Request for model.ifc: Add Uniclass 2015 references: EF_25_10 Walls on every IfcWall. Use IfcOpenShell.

First a look at what the model holds.

```python
import ifcopenshell

model = ifcopenshell.open("model.ifc")
print(model.schema)
print("classifications:", [c.Name for c in model.by_type("IfcClassification")])
for ifc_class in ("IfcDoor", "IfcRoof", "IfcStair", "IfcWall", "IfcWindow"):
    print(ifc_class, len(model.by_type(ifc_class)))
```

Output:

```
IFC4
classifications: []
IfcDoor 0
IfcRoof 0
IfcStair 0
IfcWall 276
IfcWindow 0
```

```python
import ifcopenshell
import ifcopenshell.api.classification

model = ifcopenshell.open("model.ifc")

system = ifcopenshell.api.classification.add_classification(model, classification="Uniclass 2015")

codes = {
    "IfcWall": ("EF_25_10", "Walls"),
}
for ifc_class, (code, name) in codes.items():
    products = model.by_type(ifc_class)
    ifcopenshell.api.classification.add_reference(
        model, products=products, classification=system, identification=code, name=name
    )
    print(code, len(products))

model.write("model_edited.ifc")
```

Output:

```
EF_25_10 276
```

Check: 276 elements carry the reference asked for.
